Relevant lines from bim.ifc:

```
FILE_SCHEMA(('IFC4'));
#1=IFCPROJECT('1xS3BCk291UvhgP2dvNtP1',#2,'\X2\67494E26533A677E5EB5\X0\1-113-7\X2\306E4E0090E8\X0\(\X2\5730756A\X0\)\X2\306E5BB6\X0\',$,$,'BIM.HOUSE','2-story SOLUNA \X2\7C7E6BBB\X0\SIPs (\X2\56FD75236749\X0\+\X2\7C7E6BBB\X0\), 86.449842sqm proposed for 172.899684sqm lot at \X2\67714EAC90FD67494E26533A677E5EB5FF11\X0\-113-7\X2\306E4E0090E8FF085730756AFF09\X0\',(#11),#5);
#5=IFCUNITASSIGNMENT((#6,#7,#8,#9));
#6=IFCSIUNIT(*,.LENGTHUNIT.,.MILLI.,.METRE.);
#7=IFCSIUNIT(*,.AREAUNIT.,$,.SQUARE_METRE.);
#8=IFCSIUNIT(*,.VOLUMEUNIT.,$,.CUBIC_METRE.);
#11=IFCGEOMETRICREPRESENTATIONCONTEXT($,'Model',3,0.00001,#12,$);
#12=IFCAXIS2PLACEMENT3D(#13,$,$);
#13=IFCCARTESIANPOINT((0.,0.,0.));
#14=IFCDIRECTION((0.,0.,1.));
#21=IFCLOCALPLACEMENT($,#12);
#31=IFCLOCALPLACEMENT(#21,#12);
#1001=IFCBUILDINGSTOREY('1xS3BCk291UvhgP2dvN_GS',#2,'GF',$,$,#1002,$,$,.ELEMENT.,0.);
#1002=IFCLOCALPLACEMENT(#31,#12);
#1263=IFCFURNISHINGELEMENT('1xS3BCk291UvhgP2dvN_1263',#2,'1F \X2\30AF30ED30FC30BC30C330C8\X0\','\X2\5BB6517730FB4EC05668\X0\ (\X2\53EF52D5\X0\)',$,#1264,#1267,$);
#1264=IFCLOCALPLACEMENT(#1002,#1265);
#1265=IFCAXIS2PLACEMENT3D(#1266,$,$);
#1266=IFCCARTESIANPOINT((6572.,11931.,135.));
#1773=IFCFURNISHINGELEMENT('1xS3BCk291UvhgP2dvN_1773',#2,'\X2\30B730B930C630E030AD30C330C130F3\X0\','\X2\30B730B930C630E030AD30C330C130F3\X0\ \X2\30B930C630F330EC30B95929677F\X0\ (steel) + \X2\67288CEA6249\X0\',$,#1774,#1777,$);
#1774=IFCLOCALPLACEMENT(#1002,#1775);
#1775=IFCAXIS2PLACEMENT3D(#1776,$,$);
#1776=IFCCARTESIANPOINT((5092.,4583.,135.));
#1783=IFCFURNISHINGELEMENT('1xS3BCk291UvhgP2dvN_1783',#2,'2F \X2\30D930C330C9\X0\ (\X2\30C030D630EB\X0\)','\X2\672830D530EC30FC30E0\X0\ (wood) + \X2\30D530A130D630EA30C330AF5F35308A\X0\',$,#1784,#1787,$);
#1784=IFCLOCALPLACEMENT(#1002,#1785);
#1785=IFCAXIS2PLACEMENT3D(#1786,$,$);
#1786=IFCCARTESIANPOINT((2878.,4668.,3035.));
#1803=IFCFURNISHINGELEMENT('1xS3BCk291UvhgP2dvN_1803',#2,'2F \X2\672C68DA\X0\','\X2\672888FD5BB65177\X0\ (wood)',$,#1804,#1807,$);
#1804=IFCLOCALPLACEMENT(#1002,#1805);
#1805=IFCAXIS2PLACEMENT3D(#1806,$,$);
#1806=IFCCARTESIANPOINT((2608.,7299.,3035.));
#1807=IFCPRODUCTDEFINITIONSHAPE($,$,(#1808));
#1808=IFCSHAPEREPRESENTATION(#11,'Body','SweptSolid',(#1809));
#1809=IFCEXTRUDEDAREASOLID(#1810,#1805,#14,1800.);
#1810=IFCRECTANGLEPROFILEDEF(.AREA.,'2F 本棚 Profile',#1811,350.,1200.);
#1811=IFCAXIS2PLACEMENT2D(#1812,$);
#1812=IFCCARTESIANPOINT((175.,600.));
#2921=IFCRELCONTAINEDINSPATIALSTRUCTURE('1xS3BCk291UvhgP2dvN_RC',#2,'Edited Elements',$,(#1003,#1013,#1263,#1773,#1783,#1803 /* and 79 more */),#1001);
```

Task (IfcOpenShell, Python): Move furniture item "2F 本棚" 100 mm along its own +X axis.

```python
import ifcopenshell
import ifcopenshell.api.geometry
import ifcopenshell.util.placement
import ifcopenshell.util.unit

model = ifcopenshell.open("bim.ifc")
unit_scale = ifcopenshell.util.unit.calculate_unit_scale(model)

item = model.by_guid("1xS3BCk291UvhgP2dvN_1803")
matrix = ifcopenshell.util.placement.get_local_placement(item.ObjectPlacement)
matrix[:3, 3] += matrix[:3, 0] * 0.1 / unit_scale
ifcopenshell.api.geometry.edit_object_placement(model, product=item, matrix=matrix, is_si=False)

print(ifcopenshell.util.placement.get_local_placement(item.ObjectPlacement).round(3) + 0.0)

model.write("bim-out.ifc")
```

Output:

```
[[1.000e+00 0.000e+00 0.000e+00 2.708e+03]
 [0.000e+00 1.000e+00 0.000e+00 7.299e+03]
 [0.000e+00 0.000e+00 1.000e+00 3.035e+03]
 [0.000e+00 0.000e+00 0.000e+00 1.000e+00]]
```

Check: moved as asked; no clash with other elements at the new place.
